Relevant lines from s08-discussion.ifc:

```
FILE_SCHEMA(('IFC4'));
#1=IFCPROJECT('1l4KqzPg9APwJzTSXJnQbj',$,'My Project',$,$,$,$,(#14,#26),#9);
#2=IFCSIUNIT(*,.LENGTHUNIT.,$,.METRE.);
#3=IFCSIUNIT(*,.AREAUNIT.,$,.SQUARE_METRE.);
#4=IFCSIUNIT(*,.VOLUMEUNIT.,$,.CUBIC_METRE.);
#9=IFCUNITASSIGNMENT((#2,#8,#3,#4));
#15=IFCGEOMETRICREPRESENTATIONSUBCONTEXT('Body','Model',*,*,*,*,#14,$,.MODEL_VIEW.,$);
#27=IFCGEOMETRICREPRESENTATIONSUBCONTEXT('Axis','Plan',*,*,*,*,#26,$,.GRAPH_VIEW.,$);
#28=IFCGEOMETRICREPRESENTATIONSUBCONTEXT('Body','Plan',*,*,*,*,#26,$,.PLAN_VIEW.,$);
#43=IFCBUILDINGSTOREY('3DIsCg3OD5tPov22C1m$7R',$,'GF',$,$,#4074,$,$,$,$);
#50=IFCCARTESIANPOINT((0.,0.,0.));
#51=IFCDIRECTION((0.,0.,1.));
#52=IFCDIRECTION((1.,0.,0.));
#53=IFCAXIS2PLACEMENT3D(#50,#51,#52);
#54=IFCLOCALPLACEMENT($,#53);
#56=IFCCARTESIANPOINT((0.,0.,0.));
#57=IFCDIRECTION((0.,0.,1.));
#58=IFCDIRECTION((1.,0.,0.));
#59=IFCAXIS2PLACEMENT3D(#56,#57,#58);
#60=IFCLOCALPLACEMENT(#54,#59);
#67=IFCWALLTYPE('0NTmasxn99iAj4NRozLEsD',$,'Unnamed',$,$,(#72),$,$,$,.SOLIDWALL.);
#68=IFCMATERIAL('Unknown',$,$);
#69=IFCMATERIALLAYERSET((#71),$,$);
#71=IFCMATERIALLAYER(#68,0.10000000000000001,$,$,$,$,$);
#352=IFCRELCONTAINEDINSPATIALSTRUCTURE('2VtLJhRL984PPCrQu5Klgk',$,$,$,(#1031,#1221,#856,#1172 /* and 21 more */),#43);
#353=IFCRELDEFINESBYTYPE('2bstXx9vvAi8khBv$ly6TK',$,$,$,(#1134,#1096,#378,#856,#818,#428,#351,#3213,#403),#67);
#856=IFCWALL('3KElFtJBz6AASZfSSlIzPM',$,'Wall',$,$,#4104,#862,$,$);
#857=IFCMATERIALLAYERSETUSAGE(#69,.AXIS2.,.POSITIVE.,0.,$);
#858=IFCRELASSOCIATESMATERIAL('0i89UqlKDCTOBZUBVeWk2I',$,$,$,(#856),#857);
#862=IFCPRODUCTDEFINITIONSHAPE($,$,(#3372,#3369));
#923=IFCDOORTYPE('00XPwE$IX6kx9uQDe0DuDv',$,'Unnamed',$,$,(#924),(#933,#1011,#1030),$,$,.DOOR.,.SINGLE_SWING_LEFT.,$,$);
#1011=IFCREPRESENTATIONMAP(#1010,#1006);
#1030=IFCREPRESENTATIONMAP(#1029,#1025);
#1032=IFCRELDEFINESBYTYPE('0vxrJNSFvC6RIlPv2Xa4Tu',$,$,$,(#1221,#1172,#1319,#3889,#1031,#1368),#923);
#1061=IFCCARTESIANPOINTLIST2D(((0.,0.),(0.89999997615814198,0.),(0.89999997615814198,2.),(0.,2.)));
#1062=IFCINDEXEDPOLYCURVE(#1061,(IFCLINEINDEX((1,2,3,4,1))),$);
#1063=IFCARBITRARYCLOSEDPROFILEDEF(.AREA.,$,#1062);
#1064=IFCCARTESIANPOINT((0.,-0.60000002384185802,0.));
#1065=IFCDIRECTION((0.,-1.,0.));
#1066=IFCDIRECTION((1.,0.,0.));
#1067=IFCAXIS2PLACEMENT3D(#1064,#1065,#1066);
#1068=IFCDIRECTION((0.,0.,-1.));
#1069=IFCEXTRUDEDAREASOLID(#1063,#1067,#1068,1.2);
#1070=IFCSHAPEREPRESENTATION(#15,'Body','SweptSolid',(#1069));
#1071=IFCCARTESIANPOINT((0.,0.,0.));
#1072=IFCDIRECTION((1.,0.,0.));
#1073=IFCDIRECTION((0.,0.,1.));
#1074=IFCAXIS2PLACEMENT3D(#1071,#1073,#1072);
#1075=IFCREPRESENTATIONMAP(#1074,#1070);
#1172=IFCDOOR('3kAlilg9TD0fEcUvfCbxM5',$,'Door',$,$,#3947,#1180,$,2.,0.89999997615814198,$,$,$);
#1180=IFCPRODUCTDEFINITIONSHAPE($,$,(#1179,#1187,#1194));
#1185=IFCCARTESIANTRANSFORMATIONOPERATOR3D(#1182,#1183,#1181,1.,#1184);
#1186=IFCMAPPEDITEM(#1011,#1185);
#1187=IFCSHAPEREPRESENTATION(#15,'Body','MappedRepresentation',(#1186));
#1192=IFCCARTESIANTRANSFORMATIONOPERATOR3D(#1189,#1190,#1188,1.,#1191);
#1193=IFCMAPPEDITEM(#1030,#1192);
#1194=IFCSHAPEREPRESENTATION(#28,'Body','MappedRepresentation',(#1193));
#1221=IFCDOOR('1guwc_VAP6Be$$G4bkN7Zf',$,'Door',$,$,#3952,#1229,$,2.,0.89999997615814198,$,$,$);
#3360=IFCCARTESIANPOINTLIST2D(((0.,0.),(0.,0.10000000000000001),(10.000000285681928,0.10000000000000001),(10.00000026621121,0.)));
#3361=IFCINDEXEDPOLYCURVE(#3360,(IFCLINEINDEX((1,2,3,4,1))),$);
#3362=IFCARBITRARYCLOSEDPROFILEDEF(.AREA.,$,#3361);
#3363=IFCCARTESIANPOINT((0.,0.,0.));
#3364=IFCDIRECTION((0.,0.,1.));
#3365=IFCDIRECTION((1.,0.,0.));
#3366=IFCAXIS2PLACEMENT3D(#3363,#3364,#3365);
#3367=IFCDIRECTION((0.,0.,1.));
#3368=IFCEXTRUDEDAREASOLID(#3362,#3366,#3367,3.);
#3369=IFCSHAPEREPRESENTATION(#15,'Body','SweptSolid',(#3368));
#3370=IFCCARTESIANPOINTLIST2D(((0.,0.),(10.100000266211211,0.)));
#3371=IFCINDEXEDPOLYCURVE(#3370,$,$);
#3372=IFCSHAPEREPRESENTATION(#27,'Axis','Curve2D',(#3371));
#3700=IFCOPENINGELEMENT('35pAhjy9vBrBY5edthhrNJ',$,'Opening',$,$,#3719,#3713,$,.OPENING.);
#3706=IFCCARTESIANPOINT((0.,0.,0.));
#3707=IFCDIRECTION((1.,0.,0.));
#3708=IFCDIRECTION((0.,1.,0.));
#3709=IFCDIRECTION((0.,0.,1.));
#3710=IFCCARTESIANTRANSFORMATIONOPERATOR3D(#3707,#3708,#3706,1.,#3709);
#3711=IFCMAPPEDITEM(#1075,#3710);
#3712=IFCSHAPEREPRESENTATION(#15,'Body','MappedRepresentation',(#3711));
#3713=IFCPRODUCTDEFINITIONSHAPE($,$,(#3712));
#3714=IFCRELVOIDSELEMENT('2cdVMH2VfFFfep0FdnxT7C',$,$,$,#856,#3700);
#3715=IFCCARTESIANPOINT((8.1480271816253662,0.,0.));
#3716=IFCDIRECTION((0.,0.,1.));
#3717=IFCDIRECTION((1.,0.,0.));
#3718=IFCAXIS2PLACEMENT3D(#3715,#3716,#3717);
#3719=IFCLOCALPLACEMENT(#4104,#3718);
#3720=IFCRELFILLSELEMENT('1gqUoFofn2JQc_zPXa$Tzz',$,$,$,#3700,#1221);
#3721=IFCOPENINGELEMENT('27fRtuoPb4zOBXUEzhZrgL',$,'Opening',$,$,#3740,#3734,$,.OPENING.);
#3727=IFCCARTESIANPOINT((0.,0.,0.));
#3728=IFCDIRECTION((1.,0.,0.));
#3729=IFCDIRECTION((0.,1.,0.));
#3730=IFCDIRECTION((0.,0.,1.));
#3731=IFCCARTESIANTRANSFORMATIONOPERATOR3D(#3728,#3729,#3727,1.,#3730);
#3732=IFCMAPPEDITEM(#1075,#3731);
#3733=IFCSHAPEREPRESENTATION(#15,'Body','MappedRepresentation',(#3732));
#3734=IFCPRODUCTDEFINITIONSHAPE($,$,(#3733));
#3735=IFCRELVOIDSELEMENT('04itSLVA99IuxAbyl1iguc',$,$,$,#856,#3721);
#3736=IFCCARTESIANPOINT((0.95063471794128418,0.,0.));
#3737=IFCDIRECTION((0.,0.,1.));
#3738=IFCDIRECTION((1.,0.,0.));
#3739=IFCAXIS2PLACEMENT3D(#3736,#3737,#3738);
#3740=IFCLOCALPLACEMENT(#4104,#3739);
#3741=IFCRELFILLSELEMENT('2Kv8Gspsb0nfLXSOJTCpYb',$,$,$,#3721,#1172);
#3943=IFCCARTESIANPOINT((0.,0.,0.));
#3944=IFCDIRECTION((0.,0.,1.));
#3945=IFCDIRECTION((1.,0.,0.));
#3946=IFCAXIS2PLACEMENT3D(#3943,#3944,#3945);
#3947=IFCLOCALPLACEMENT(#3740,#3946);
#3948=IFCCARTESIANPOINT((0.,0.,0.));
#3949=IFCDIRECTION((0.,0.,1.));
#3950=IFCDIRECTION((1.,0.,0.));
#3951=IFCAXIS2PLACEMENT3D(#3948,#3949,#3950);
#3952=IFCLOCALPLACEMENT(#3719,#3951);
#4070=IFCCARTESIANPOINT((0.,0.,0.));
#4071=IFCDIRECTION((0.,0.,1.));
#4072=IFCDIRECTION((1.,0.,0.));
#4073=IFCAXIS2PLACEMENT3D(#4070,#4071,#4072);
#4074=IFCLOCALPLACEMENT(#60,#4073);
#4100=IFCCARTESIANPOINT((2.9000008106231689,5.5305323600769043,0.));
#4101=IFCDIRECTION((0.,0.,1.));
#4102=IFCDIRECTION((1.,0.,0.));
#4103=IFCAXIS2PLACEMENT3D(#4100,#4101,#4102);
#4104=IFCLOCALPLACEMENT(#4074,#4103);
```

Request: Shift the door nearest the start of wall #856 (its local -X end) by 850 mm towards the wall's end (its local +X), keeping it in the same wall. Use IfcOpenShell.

```python
import ifcopenshell
import ifcopenshell.api.geometry
import ifcopenshell.util.placement

model = ifcopenshell.open("s08-discussion.ifc")

door = model.by_guid("3kAlilg9TD0fEcUvfCbxM5")
opening = door.FillsVoids[0].RelatingOpeningElement
wall = opening.VoidsElements[0].RelatingBuildingElement

wall_matrix = ifcopenshell.util.placement.get_local_placement(wall.ObjectPlacement)
shift = wall_matrix[:3, 0] * 0.85
before = ifcopenshell.util.placement.get_local_placement(door.ObjectPlacement)[:3, 3].copy()

# The door is placed relative to its opening, so it follows when the opening moves.
matrix = ifcopenshell.util.placement.get_local_placement(opening.ObjectPlacement)
matrix[:3, 3] += shift
ifcopenshell.api.geometry.edit_object_placement(
    model, product=opening, matrix=matrix, is_si=False, should_transform_children=True
)

after = ifcopenshell.util.placement.get_local_placement(door.ObjectPlacement)[:3, 3]
print("door moved by", (after - before).round(3) + 0.0)

model.write("s08-discussion_edited.ifc")
```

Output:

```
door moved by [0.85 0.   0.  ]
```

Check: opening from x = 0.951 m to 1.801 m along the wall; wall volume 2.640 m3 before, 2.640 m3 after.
